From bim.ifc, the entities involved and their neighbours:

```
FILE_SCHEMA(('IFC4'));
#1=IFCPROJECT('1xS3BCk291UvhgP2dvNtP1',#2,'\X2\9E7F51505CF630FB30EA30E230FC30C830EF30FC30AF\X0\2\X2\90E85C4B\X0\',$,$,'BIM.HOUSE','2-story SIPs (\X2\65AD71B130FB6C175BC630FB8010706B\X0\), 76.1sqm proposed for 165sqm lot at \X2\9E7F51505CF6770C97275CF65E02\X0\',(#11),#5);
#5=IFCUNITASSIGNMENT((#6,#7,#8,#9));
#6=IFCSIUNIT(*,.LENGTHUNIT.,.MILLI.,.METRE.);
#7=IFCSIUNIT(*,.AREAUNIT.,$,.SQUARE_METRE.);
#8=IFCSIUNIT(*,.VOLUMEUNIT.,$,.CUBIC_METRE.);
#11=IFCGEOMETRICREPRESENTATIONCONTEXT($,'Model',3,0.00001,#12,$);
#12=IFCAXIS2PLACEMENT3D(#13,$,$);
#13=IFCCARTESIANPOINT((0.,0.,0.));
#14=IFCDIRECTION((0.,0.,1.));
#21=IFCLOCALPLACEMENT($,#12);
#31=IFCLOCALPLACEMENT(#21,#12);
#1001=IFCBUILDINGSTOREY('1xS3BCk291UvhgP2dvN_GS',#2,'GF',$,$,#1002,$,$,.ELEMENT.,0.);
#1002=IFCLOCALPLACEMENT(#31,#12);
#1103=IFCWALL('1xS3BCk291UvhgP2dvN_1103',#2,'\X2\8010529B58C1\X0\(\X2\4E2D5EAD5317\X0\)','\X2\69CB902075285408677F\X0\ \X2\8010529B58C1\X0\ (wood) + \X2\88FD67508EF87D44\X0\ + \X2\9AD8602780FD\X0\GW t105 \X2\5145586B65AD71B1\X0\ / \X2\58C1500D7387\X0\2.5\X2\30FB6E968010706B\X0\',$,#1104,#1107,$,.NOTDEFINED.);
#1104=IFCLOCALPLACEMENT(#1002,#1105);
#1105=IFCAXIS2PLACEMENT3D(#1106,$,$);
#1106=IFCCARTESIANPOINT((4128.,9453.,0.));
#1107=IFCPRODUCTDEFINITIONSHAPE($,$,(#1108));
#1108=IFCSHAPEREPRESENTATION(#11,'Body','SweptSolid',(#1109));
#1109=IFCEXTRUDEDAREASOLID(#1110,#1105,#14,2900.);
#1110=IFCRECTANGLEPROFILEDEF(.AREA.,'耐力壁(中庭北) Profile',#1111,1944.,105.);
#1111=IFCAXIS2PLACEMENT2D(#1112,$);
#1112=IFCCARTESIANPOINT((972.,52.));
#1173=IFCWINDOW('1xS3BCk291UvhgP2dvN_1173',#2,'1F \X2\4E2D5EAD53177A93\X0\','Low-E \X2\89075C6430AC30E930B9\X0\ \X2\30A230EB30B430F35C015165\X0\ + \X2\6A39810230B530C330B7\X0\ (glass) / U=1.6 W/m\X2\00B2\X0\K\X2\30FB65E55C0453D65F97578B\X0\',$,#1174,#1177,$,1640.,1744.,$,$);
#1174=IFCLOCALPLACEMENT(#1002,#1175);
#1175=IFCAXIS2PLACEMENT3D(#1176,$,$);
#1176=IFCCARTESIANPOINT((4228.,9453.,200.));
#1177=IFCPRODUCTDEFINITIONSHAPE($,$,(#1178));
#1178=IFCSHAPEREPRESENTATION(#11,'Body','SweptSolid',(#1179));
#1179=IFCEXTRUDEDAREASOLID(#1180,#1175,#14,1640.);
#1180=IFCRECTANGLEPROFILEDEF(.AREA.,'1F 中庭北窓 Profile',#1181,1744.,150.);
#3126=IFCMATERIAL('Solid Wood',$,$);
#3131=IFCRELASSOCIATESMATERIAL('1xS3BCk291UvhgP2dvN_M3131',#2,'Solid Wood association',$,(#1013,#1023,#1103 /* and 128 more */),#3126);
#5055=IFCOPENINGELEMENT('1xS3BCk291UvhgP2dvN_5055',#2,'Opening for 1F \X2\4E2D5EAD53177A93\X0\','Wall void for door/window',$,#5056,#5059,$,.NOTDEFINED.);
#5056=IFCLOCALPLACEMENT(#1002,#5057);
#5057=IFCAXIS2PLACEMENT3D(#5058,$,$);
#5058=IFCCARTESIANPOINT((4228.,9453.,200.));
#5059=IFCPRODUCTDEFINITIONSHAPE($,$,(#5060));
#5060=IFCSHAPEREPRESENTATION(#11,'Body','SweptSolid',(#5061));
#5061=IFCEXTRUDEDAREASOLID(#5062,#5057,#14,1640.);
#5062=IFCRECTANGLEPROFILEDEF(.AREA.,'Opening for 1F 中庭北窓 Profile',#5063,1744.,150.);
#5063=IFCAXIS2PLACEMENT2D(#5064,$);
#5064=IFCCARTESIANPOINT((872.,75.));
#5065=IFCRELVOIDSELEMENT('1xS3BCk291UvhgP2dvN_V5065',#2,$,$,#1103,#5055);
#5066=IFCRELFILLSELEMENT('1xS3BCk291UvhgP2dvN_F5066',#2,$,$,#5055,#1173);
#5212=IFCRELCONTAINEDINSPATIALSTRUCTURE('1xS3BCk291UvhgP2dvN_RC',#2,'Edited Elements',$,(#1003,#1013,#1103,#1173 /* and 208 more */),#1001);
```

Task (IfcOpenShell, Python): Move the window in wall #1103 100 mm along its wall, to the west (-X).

```python
import ifcopenshell
import ifcopenshell.api.geometry
import ifcopenshell.util.placement
import ifcopenshell.util.unit

model = ifcopenshell.open("bim.ifc")
unit_scale = ifcopenshell.util.unit.calculate_unit_scale(model)

window = model.by_guid("1xS3BCk291UvhgP2dvN_1173")
opening = window.FillsVoids[0].RelatingOpeningElement
wall = opening.VoidsElements[0].RelatingBuildingElement

wall_matrix = ifcopenshell.util.placement.get_local_placement(wall.ObjectPlacement)
shift = wall_matrix[:3, 0] * -0.1 / unit_scale
before = ifcopenshell.util.placement.get_local_placement(window.ObjectPlacement)[:3, 3].copy()

# The window is not placed relative to its opening, so move both.
for product in (opening, window):
    matrix = ifcopenshell.util.placement.get_local_placement(product.ObjectPlacement)
    matrix[:3, 3] += shift
    ifcopenshell.api.geometry.edit_object_placement(model, product=product, matrix=matrix, is_si=False)

after = ifcopenshell.util.placement.get_local_placement(window.ObjectPlacement)[:3, 3]
print("window moved by", (after - before).round(3) + 0.0)

model.write("bim_rev.ifc")
```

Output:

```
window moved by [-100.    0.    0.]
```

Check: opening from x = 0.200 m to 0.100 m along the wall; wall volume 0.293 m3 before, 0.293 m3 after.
